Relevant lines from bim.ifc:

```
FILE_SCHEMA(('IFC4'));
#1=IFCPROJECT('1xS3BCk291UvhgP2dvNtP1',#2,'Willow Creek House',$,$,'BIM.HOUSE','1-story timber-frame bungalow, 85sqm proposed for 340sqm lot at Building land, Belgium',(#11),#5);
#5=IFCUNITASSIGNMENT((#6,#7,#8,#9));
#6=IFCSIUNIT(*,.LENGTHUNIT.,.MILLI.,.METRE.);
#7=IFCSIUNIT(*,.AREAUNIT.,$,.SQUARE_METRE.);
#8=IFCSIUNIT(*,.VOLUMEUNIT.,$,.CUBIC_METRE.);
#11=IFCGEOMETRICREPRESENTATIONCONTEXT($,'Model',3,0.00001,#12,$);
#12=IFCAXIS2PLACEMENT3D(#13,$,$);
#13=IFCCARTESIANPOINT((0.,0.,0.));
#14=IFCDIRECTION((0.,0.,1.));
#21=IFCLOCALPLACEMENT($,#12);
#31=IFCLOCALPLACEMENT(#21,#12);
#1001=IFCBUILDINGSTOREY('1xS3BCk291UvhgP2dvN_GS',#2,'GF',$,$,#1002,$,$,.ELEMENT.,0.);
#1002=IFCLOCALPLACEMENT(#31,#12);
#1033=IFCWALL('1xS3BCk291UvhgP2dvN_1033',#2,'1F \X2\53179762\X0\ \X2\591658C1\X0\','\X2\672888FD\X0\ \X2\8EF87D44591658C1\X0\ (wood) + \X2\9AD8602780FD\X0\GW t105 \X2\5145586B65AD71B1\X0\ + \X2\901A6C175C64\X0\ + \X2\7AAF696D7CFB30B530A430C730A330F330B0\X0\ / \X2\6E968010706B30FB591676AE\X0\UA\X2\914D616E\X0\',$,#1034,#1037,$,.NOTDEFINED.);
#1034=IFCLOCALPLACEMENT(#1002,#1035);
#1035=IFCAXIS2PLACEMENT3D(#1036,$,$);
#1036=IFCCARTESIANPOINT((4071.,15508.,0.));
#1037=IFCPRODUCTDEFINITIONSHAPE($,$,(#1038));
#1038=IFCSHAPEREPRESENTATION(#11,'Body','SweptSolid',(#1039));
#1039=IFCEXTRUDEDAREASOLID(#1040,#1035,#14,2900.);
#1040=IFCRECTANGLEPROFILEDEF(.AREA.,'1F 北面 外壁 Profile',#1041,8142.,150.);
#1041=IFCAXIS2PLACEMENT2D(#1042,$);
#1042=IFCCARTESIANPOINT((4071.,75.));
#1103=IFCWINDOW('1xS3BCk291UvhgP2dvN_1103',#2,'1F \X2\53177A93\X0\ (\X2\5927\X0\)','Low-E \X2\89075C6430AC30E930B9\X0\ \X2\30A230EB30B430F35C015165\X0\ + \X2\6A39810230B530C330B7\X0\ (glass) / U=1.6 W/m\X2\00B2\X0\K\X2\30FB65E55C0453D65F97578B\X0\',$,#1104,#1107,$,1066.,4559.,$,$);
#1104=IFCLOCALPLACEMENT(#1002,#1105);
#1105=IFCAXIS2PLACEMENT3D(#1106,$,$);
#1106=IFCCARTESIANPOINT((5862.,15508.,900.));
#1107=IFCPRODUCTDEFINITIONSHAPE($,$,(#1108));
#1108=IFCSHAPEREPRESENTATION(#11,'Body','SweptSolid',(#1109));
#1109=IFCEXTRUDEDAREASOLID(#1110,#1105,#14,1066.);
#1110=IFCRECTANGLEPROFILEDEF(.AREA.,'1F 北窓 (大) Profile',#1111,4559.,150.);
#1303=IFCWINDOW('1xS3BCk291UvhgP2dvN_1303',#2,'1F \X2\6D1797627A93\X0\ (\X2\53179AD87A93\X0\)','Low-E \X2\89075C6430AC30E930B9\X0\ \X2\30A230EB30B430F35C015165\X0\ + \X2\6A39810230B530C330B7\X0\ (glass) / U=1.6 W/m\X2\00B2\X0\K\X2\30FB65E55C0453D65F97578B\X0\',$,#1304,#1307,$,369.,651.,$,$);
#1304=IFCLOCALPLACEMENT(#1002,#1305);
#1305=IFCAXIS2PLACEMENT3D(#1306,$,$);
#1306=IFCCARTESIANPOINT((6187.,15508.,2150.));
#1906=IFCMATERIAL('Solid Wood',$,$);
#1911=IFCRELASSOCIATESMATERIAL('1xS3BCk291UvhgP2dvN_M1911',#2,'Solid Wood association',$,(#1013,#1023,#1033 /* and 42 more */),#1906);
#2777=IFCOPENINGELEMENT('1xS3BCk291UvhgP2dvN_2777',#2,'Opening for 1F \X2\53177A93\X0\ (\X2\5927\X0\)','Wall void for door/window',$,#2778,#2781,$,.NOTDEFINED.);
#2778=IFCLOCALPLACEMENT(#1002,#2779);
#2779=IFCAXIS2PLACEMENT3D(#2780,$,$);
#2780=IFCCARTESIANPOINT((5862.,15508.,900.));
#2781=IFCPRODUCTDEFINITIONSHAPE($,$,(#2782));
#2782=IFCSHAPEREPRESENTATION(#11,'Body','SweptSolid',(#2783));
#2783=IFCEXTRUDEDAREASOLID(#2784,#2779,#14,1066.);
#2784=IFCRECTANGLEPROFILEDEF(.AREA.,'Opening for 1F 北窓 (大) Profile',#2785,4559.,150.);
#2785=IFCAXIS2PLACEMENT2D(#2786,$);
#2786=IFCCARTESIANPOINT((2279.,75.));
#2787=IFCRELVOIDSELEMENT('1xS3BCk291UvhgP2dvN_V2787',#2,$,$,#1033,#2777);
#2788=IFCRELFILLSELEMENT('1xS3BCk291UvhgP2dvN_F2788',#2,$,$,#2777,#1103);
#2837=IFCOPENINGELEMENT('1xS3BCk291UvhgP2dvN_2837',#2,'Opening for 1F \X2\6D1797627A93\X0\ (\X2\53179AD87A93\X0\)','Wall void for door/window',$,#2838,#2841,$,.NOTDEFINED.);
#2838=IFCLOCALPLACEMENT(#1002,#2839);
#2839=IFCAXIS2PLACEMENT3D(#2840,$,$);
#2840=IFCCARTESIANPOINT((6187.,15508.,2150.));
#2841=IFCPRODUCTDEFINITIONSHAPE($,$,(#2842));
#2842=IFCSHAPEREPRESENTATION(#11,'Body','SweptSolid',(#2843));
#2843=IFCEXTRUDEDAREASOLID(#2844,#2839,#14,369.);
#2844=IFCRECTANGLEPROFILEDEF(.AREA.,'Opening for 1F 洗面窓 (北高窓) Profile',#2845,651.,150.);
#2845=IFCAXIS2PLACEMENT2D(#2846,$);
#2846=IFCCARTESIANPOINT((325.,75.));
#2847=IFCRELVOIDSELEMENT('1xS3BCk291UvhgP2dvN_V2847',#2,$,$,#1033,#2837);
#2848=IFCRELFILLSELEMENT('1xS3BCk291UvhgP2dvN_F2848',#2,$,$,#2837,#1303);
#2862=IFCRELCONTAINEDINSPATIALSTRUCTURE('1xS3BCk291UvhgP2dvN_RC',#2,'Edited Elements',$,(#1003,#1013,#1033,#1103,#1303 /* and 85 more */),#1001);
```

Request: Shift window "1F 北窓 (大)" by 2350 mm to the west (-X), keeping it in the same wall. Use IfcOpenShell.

```python
import ifcopenshell
import ifcopenshell.api.geometry
import ifcopenshell.util.placement
import ifcopenshell.util.unit

model = ifcopenshell.open("bim.ifc")
unit_scale = ifcopenshell.util.unit.calculate_unit_scale(model)

window = model.by_id(1103)
opening = window.FillsVoids[0].RelatingOpeningElement
wall = opening.VoidsElements[0].RelatingBuildingElement

wall_matrix = ifcopenshell.util.placement.get_local_placement(wall.ObjectPlacement)
shift = wall_matrix[:3, 0] * -2.35 / unit_scale
before = ifcopenshell.util.placement.get_local_placement(window.ObjectPlacement)[:3, 3].copy()

# The window is not placed relative to its opening, so move both.
for product in (opening, window):
    matrix = ifcopenshell.util.placement.get_local_placement(product.ObjectPlacement)
    matrix[:3, 3] += shift
    ifcopenshell.api.geometry.edit_object_placement(model, product=product, matrix=matrix, is_si=False)

after = ifcopenshell.util.placement.get_local_placement(window.ObjectPlacement)[:3, 3]
print("window moved by", (after - before).round(3) + 0.0)

model.write("bim_edited.ifc")
```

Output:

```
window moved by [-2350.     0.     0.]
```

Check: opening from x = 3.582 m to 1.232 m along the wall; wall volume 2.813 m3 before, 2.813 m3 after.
